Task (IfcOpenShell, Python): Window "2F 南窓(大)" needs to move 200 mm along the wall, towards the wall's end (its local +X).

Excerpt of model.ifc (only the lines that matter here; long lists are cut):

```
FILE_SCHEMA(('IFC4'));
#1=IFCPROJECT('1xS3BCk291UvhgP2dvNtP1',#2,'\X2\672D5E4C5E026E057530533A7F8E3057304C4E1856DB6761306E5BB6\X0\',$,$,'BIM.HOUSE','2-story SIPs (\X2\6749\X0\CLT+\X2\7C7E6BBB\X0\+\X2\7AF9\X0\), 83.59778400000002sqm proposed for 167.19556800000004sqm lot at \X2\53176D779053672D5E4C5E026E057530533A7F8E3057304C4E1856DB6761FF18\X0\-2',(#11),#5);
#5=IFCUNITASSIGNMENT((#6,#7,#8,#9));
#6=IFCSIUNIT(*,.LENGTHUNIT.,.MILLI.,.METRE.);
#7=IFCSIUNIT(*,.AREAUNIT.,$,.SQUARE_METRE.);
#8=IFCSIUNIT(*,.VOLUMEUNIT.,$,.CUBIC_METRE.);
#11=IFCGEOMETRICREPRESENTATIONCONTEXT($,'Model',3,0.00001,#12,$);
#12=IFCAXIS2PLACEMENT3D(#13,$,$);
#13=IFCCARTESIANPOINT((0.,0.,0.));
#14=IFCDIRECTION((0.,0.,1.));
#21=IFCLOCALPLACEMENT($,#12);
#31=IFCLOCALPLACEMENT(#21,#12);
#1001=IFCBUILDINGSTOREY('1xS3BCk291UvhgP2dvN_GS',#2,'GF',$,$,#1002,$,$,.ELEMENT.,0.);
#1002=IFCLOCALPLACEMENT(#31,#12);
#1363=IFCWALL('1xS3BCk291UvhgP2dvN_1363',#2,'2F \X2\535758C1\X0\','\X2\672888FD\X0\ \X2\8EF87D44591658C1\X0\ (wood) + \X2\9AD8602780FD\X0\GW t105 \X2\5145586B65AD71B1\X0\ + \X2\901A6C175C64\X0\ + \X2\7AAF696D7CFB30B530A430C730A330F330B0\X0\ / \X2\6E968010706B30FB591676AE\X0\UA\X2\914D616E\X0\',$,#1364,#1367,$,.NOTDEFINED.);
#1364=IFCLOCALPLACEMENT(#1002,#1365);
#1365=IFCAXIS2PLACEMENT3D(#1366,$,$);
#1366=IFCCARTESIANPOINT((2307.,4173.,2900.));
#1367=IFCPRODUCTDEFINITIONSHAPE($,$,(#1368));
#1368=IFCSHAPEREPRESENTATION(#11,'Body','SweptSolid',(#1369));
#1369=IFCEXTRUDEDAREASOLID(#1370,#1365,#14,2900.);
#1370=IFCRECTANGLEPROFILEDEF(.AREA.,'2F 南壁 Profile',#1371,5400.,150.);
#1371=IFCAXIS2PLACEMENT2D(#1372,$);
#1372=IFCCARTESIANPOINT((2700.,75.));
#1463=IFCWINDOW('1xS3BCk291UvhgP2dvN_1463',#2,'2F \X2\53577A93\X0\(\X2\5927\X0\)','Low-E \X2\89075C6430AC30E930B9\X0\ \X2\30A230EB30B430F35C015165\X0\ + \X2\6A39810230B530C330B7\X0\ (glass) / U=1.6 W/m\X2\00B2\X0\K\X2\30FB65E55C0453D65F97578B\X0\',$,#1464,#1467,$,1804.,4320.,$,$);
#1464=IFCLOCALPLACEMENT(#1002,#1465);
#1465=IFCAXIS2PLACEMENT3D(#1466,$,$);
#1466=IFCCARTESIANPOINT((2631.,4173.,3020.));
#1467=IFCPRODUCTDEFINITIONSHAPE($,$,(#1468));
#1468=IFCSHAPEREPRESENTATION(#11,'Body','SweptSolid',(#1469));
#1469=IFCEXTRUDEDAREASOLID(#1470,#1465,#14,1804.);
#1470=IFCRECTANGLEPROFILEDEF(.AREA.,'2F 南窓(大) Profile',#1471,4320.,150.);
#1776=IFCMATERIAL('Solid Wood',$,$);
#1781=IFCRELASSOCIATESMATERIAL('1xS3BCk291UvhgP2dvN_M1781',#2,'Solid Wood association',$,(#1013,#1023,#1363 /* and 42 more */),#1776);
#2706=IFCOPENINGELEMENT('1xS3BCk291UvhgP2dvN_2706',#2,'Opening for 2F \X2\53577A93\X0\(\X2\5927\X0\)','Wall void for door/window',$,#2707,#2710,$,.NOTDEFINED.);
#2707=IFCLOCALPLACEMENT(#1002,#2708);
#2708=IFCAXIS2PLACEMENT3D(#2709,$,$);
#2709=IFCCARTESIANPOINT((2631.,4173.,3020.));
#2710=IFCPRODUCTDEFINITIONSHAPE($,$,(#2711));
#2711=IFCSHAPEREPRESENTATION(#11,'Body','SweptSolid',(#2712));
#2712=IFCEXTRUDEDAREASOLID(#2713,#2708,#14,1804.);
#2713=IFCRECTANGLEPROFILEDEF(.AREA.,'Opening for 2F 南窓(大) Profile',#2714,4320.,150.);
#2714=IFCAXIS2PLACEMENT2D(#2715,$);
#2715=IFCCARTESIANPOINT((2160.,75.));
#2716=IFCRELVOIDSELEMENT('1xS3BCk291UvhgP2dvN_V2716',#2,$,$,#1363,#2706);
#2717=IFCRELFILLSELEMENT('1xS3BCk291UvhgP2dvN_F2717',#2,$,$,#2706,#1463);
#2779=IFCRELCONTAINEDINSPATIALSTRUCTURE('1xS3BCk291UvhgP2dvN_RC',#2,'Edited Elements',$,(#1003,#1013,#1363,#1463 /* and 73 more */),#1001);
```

```python
import ifcopenshell
import ifcopenshell.api.geometry
import ifcopenshell.util.placement

model = ifcopenshell.open("model.ifc")

window = model.by_guid("1xS3BCk291UvhgP2dvN_1463")
opening = window.FillsVoids[0].RelatingOpeningElement
wall = opening.VoidsElements[0].RelatingBuildingElement

wall_matrix = ifcopenshell.util.placement.get_local_placement(wall.ObjectPlacement)
shift = wall_matrix[:3, 0] * 200.0
before = ifcopenshell.util.placement.get_local_placement(window.ObjectPlacement)[:3, 3].copy()

# The window is not placed relative to its opening, so move both.
for product in (opening, window):
    matrix = ifcopenshell.util.placement.get_local_placement(product.ObjectPlacement)
    matrix[:3, 3] += shift
    ifcopenshell.api.geometry.edit_object_placement(model, product=product, matrix=matrix, is_si=False)

after = ifcopenshell.util.placement.get_local_placement(window.ObjectPlacement)[:3, 3]
print("window moved by", (after - before).round(3) + 0.0)

model.write("model_rev.ifc")
```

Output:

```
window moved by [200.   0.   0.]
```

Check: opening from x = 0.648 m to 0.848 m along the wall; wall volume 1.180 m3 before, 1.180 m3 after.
